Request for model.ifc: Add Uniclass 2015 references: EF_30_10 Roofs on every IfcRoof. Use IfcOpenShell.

First a look at what the model holds.

```python
import ifcopenshell

model = ifcopenshell.open("model.ifc")
print(model.schema)
print("classifications:", [c.Name for c in model.by_type("IfcClassification")])
for ifc_class in ("IfcDoor", "IfcRoof", "IfcStair", "IfcWall", "IfcWindow"):
    print(ifc_class, len(model.by_type(ifc_class)))
```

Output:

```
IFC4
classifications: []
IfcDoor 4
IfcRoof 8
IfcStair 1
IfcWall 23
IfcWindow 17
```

```python
import ifcopenshell
import ifcopenshell.api.classification

model = ifcopenshell.open("model.ifc")

system = ifcopenshell.api.classification.add_classification(model, classification="Uniclass 2015")

codes = {
    "IfcRoof": ("EF_30_10", "Roofs"),
}
for ifc_class, (code, name) in codes.items():
    products = model.by_type(ifc_class)
    ifcopenshell.api.classification.add_reference(
        model, products=products, classification=system, identification=code, name=name
    )
    print(code, len(products))

model.write("model_v2.ifc")
```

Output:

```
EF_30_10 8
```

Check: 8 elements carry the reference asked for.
